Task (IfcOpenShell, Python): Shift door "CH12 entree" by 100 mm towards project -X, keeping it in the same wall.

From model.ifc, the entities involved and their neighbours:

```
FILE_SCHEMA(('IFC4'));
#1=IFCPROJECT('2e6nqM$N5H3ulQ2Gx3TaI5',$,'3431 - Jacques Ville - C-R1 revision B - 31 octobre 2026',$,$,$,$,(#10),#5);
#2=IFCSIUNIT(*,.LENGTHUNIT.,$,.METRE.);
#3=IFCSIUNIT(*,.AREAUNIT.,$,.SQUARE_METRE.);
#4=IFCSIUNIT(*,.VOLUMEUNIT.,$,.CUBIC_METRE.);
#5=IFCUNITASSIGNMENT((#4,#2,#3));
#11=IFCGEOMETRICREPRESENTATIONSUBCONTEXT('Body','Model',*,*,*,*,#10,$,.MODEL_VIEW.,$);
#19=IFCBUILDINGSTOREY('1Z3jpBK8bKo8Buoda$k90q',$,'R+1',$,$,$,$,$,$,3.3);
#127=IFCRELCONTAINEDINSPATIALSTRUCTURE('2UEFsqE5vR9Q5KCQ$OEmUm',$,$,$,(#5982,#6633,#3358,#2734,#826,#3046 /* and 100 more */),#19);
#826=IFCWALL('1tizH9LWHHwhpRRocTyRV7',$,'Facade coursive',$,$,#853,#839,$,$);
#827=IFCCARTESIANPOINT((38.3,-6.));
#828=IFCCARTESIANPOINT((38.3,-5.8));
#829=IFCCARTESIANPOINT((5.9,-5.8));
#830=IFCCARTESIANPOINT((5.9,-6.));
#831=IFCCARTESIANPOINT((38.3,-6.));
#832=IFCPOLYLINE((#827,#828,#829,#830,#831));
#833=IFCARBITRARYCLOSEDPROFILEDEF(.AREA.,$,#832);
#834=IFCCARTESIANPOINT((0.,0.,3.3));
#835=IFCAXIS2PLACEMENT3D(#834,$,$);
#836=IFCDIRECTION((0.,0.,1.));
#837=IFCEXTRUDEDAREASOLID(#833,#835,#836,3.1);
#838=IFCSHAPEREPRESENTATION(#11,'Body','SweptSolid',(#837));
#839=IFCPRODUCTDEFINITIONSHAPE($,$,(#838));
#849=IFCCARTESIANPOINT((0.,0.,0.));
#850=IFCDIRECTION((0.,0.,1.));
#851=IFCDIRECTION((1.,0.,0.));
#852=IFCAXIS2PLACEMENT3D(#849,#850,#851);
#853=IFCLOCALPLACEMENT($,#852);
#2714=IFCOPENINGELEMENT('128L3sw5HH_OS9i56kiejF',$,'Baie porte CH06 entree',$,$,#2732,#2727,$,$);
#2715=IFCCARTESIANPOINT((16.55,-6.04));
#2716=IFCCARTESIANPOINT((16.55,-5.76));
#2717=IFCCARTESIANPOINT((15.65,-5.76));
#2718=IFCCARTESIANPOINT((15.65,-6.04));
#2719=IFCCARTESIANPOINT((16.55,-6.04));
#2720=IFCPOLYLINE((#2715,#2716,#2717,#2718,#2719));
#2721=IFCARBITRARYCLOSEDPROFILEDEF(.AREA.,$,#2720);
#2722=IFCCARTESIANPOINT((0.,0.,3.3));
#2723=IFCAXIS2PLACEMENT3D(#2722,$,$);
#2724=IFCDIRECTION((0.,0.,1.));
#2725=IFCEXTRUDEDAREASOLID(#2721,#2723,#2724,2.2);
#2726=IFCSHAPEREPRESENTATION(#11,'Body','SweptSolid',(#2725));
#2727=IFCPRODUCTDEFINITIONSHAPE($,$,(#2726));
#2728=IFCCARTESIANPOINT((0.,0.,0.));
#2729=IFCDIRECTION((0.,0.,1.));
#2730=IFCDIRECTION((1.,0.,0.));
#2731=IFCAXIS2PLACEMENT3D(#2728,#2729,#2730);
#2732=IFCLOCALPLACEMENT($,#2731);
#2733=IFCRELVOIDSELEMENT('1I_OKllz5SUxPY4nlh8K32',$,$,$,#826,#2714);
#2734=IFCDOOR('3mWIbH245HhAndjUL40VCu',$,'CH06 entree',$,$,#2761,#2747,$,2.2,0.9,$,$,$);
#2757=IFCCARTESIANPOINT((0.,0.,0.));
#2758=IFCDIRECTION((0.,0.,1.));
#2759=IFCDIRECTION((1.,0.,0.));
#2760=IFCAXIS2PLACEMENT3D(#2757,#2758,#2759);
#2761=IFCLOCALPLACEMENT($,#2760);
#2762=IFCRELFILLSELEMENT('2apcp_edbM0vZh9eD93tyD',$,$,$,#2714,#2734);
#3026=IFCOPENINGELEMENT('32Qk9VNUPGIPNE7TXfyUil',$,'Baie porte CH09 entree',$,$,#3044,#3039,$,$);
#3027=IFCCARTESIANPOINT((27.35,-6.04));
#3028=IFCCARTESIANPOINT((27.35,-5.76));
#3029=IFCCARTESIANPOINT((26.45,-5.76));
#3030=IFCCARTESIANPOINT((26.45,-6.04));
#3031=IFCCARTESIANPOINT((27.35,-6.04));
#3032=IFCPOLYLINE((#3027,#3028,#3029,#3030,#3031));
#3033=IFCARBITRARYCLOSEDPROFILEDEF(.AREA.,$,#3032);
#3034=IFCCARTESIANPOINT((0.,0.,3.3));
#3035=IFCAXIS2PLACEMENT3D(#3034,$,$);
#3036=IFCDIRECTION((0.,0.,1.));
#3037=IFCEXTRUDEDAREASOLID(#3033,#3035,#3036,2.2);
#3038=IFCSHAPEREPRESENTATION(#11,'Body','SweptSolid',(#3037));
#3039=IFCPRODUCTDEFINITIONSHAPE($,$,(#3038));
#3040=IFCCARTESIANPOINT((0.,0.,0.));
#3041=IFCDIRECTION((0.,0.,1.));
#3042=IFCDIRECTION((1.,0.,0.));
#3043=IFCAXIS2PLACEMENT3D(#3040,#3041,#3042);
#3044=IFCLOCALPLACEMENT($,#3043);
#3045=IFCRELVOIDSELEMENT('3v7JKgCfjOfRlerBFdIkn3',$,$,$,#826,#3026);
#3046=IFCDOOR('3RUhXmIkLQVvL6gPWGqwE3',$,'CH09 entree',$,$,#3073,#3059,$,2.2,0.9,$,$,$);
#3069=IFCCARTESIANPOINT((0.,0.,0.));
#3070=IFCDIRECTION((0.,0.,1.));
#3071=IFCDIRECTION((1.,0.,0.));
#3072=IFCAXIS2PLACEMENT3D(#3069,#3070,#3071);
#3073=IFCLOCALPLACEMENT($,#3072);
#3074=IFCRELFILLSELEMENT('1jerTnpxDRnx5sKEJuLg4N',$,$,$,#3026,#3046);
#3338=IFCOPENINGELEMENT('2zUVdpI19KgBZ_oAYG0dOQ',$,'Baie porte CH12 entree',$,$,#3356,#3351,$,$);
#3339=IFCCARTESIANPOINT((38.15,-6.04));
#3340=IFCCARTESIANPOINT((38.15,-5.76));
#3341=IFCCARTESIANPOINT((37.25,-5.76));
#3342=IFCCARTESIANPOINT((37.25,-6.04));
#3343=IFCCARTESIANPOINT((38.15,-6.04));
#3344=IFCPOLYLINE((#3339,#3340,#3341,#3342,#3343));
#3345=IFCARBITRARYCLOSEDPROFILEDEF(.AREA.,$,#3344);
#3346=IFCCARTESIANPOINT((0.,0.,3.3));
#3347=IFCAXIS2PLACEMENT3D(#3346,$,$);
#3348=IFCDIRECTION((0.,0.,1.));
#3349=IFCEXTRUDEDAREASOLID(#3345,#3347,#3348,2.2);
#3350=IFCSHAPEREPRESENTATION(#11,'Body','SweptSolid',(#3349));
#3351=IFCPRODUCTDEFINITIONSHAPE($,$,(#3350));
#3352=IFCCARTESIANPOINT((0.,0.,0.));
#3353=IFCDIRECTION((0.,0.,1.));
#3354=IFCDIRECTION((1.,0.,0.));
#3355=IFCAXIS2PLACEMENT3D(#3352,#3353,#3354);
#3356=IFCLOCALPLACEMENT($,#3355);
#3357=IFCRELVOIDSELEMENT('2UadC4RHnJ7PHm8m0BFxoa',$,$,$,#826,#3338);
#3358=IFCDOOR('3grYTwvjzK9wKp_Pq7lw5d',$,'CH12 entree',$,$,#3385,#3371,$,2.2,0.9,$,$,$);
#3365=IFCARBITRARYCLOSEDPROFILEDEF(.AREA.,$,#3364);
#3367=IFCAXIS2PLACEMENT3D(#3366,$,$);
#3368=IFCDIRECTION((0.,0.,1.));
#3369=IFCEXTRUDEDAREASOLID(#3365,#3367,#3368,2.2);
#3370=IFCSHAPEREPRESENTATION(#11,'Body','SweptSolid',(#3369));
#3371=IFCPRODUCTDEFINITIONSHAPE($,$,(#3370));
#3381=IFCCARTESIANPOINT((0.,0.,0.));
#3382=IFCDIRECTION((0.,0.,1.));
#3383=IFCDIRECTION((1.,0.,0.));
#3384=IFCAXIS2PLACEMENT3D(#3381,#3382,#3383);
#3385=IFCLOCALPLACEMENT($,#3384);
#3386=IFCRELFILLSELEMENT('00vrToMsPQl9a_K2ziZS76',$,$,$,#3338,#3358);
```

```python
import ifcopenshell
import ifcopenshell.api.geometry
import ifcopenshell.util.placement

model = ifcopenshell.open("model.ifc")

door = model.by_id(3358)
opening = door.FillsVoids[0].RelatingOpeningElement
wall = opening.VoidsElements[0].RelatingBuildingElement

wall_matrix = ifcopenshell.util.placement.get_local_placement(wall.ObjectPlacement)
shift = wall_matrix[:3, 0] * -0.1
before = ifcopenshell.util.placement.get_local_placement(door.ObjectPlacement)[:3, 3].copy()

# The door is not placed relative to its opening, so move both.
for product in (opening, door):
    matrix = ifcopenshell.util.placement.get_local_placement(product.ObjectPlacement)
    matrix[:3, 3] += shift
    ifcopenshell.api.geometry.edit_object_placement(model, product=product, matrix=matrix, is_si=False)

after = ifcopenshell.util.placement.get_local_placement(door.ObjectPlacement)[:3, 3]
print("door moved by", (after - before).round(3) + 0.0)

model.write("model_updated.ifc")
```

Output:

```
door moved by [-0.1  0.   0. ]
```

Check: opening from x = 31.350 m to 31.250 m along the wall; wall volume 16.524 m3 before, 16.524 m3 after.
